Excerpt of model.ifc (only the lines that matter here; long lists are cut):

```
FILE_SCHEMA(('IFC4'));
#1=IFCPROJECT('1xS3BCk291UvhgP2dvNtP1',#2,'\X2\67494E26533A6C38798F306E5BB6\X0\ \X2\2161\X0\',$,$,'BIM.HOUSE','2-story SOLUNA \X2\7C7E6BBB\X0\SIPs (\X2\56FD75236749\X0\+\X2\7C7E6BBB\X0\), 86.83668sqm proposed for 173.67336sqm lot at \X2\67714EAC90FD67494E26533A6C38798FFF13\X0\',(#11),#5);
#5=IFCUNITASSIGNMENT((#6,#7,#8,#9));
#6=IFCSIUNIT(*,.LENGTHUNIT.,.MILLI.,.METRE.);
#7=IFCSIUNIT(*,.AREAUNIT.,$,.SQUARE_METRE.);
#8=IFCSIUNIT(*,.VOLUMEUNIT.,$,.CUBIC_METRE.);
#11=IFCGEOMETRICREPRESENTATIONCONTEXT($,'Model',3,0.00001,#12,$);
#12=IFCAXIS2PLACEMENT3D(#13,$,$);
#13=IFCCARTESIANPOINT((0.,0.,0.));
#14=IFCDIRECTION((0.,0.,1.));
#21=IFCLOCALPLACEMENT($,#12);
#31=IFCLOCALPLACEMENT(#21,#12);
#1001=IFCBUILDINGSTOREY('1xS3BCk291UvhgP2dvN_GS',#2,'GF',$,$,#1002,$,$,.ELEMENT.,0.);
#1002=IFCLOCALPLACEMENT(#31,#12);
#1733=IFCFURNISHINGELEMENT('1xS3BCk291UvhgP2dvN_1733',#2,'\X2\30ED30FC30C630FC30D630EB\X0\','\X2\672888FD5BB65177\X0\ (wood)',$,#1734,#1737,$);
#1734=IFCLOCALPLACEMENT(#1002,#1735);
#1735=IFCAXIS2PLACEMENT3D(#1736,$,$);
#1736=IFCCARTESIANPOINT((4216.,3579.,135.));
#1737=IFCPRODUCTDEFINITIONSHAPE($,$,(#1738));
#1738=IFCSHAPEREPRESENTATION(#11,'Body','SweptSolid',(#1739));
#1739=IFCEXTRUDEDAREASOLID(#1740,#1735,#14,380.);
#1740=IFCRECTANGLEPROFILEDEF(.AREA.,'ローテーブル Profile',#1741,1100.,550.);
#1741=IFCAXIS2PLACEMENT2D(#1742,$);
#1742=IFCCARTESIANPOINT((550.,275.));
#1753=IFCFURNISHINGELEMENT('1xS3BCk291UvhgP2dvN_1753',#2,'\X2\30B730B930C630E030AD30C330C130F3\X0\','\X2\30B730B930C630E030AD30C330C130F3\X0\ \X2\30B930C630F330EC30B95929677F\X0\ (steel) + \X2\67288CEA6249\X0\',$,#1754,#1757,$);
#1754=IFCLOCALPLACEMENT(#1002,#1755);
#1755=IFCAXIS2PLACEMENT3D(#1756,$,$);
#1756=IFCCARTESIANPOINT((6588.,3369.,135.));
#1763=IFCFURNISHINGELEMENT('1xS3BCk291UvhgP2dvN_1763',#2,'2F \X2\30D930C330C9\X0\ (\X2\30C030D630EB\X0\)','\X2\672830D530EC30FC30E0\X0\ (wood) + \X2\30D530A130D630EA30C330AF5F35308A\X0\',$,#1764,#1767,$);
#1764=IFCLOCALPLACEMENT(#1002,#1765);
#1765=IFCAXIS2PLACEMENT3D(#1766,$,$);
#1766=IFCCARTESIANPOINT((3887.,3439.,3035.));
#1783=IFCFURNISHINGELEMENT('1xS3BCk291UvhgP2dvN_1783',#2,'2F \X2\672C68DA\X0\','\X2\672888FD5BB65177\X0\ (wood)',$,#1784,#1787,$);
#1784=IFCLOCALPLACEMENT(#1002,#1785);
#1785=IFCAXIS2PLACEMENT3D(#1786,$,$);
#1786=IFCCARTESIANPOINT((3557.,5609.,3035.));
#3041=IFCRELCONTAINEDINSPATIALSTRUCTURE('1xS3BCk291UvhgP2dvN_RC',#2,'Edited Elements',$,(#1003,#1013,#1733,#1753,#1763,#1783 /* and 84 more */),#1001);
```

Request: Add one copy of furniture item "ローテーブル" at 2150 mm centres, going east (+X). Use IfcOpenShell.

```python
import numpy as np
import ifcopenshell
import ifcopenshell.api.geometry
import ifcopenshell.api.root
import ifcopenshell.util.element
import ifcopenshell.util.placement
import ifcopenshell.util.unit

model = ifcopenshell.open("model.ifc")
unit_scale = ifcopenshell.util.unit.calculate_unit_scale(model)


def reuse_history(source, copy):
    """copy_class also copies each property set's owner history, people and application; keep the originals."""
    for rel in copy.IsDefinedBy:
        if rel.is_a("IfcRelDefinesByProperties") and (history := rel.RelatingPropertyDefinition.OwnerHistory):
            rel.RelatingPropertyDefinition.OwnerHistory = source.OwnerHistory
            ifcopenshell.util.element.remove_deep2(model, history)


source = model.by_guid("1xS3BCk291UvhgP2dvN_1733")
base = ifcopenshell.util.placement.get_local_placement(source.ObjectPlacement)
step = np.array([1.0, 0.0, 0.0]) * 2.15 / unit_scale

for i in range(1, 2):
    copy = ifcopenshell.api.root.copy_class(model, product=source)
    copy.Representation = ifcopenshell.util.element.copy_deep(
        model, source.Representation, exclude=["IfcGeometricRepresentationContext", "IfcRepresentationMap"]
    )
    reuse_history(source, copy)
    matrix = base.copy()
    matrix[:3, 3] += i * step
    print("added at", matrix[:3, 3].round(3) + 0.0)
    ifcopenshell.api.geometry.edit_object_placement(model, product=copy, matrix=matrix, is_si=False)

model.write("model_v2.ifc")
```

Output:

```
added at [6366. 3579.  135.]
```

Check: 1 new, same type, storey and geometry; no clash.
